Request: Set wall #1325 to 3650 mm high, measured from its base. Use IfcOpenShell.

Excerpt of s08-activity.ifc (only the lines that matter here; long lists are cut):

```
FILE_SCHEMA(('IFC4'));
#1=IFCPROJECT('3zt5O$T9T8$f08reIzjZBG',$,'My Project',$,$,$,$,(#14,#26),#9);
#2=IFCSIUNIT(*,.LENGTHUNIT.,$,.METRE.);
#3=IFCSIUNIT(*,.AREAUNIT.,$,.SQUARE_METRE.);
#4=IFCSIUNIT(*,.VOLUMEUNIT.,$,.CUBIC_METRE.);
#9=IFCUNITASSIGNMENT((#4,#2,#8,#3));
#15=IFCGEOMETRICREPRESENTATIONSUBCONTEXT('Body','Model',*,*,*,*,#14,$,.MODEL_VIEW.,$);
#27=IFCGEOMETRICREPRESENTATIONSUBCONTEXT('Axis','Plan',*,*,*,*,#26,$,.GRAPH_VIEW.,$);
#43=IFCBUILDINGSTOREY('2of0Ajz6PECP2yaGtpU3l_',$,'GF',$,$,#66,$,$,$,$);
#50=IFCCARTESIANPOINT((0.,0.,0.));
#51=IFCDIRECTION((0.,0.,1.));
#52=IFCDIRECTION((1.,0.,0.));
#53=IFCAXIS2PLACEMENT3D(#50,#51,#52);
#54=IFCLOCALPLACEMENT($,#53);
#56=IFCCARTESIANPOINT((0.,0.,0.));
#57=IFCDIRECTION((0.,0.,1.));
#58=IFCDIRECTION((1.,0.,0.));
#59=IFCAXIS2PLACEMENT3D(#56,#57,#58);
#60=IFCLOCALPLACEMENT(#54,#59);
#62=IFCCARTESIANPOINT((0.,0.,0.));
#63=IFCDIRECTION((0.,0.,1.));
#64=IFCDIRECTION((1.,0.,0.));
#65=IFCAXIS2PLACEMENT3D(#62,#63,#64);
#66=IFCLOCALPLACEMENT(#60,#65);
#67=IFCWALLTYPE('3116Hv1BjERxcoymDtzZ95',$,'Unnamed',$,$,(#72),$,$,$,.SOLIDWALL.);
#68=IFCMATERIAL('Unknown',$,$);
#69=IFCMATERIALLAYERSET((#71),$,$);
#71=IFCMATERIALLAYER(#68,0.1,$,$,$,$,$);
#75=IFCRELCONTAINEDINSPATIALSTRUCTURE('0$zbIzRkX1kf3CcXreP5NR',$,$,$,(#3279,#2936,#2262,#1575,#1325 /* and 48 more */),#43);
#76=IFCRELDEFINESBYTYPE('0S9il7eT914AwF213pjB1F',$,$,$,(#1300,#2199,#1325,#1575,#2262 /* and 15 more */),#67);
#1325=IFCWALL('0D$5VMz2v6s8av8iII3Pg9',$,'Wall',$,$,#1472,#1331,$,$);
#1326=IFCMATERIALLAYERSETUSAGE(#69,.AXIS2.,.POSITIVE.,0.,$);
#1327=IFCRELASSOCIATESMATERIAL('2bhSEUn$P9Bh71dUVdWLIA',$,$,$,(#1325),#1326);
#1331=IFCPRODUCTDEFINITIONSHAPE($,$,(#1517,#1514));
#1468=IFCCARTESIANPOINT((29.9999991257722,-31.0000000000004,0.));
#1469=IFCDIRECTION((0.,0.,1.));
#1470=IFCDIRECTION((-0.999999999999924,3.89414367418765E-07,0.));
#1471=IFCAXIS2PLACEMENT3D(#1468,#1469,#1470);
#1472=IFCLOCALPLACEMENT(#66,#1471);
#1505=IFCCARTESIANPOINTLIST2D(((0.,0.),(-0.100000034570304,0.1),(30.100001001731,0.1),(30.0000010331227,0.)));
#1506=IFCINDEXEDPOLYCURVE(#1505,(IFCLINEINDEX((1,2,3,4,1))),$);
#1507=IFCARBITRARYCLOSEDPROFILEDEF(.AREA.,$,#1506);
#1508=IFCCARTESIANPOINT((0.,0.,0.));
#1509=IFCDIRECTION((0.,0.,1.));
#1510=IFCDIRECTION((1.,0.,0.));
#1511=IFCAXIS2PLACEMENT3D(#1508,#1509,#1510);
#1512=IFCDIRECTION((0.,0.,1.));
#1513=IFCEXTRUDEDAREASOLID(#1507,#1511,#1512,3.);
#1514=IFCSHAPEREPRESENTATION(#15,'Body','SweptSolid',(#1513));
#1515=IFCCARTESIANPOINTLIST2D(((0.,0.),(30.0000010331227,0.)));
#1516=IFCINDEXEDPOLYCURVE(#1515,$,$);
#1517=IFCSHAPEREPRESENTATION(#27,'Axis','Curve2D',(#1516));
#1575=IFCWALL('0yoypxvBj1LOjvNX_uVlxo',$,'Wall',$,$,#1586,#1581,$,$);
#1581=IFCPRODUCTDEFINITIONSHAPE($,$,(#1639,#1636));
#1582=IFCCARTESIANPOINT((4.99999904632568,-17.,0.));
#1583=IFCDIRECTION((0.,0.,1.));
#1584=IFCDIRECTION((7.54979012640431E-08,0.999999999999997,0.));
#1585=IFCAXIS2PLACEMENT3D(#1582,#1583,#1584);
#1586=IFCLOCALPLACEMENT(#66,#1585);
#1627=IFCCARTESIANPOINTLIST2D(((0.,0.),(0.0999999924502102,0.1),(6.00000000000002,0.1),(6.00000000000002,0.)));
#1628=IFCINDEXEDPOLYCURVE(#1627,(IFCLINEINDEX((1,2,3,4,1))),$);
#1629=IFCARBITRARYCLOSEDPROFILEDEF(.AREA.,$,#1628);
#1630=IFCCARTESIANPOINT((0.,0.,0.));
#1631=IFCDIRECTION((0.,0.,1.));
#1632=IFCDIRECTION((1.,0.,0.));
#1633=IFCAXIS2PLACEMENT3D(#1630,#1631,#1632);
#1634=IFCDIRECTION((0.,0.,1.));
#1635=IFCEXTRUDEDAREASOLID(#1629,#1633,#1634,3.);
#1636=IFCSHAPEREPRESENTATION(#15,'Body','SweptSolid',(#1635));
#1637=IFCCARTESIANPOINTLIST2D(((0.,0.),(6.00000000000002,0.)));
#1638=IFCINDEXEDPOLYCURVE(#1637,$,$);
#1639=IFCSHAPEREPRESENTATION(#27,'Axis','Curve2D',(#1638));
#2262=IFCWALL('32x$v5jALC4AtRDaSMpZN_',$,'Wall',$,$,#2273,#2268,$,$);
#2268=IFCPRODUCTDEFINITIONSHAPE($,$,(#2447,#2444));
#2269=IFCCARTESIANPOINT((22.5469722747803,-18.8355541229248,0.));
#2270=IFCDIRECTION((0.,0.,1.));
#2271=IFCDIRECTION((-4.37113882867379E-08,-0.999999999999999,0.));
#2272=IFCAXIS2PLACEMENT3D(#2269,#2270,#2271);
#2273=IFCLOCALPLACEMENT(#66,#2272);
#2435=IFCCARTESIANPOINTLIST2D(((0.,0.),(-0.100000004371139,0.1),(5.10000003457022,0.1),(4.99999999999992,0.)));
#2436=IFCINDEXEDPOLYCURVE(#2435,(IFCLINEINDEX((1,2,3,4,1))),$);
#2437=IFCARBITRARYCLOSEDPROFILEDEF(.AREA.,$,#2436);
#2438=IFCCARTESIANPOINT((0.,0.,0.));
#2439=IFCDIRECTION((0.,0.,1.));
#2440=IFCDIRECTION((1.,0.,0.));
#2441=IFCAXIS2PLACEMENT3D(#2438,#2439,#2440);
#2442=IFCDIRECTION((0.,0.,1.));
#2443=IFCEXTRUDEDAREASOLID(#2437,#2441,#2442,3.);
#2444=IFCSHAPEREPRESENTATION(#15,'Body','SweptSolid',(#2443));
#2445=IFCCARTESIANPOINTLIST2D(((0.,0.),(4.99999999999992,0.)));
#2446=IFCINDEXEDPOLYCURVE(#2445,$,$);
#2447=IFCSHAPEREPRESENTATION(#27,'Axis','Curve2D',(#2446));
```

```python
import ifcopenshell
import ifcopenshell.geom
import ifcopenshell.util.representation
import ifcopenshell.util.shape
import ifcopenshell.util.unit

model = ifcopenshell.open("s08-activity.ifc")
unit_scale = ifcopenshell.util.unit.calculate_unit_scale(model)
settings = ifcopenshell.geom.settings()


def volume(element):
    """Net volume in cubic metres, openings subtracted."""
    shape = ifcopenshell.geom.create_shape(settings, element)
    return ifcopenshell.util.shape.get_volume(shape.geometry)


wall = model.by_guid("0D$5VMz2v6s8av8iII3Pg9")
before = volume(wall)

body = ifcopenshell.util.representation.get_representation(wall, "Model", "Body")
solid = body.Items[0]
old_height = solid.Depth
solid.Depth = 3.65 / unit_scale
after = volume(wall)

print(f"height {old_height:g} -> {solid.Depth:g}, volume {before:.3f} -> {after:.3f} m3")

model.write("s08-activity_v2.ifc")
```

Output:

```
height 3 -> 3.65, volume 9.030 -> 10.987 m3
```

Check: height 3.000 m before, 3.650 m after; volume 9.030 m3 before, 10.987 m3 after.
